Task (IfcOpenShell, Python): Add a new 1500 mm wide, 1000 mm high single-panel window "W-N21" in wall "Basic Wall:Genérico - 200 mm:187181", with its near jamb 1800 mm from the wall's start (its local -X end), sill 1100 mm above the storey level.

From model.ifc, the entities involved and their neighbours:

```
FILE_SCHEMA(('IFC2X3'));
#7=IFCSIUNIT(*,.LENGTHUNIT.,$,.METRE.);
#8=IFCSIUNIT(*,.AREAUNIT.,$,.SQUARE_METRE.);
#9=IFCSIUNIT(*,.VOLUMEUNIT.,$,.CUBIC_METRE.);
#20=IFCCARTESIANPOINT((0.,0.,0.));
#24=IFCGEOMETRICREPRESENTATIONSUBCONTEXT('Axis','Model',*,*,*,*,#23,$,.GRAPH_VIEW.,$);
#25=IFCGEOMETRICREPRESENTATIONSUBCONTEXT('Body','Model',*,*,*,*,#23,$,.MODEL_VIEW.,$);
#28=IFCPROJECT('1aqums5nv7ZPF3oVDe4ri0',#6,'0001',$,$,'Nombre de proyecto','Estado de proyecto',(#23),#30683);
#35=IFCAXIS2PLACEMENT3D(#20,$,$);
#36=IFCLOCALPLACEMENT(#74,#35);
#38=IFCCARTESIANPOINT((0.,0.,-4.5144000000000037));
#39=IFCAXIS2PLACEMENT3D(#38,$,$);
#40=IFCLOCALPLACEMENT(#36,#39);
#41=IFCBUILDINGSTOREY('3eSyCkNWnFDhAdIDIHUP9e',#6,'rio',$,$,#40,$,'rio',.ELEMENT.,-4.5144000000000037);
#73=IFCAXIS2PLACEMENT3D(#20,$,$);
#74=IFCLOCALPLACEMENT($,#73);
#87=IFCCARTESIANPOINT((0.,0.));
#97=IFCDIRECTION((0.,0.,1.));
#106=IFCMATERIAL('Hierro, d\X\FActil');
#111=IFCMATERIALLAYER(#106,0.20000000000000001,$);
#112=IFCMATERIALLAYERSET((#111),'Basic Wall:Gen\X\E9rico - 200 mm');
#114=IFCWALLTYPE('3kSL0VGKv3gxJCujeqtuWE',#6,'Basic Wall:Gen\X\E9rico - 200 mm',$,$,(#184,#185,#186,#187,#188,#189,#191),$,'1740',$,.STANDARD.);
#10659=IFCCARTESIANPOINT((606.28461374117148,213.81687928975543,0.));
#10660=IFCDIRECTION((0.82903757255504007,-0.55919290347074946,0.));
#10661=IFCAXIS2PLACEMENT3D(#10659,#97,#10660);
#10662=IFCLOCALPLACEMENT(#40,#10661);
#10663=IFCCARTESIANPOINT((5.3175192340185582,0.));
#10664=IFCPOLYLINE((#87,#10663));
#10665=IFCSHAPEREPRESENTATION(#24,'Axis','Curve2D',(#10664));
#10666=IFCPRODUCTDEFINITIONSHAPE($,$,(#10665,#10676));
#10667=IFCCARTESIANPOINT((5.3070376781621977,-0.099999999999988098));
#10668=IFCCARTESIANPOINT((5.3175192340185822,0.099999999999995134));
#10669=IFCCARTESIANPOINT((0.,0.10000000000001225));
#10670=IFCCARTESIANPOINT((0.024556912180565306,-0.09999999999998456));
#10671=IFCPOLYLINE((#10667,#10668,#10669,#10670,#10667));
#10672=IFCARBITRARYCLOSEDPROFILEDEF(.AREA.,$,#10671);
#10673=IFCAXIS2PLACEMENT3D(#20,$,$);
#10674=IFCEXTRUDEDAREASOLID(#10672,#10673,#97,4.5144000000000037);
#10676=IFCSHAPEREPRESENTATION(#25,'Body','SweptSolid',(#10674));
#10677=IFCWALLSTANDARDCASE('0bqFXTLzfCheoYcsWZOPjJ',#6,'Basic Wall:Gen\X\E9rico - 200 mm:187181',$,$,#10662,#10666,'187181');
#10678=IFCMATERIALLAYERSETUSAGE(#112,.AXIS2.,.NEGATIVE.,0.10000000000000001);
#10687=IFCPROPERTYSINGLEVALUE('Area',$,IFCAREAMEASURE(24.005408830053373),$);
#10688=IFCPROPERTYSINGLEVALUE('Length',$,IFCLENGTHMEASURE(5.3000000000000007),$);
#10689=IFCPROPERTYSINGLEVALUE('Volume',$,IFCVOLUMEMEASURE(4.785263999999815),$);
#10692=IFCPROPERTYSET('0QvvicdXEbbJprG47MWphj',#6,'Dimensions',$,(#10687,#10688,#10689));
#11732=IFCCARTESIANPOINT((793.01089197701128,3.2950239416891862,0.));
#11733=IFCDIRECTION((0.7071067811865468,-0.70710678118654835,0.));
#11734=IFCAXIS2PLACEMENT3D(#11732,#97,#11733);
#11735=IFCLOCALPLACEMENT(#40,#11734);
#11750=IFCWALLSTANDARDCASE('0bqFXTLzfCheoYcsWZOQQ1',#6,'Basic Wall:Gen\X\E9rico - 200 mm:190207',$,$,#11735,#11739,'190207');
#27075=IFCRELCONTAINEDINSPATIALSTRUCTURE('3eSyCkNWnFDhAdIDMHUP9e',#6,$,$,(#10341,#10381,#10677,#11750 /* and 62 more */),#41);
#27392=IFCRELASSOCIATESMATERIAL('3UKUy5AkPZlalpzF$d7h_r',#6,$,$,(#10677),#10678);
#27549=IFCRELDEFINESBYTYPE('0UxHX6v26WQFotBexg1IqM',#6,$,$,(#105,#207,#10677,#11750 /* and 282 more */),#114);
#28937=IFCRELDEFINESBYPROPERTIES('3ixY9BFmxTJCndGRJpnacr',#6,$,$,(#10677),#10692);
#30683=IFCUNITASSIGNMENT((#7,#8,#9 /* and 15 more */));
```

```python
import numpy as np
import ifcopenshell
import ifcopenshell.api.feature
import ifcopenshell.api.geometry
import ifcopenshell.api.pset
import ifcopenshell.api.root
import ifcopenshell.api.spatial
import ifcopenshell.api.type
import ifcopenshell.geom
import ifcopenshell.util.element
import ifcopenshell.util.placement
import ifcopenshell.util.representation
import ifcopenshell.util.shape
import ifcopenshell.util.unit

model = ifcopenshell.open("model.ifc")
unit_scale = ifcopenshell.util.unit.calculate_unit_scale(model)
area_scale = ifcopenshell.util.unit.calculate_unit_scale(model, "AREAUNIT")
volume_scale = ifcopenshell.util.unit.calculate_unit_scale(model, "VOLUMEUNIT")
settings = ifcopenshell.geom.settings()


def volume(element):
    """Net volume in cubic metres, openings subtracted."""
    shape = ifcopenshell.geom.create_shape(settings, element)
    return ifcopenshell.util.shape.get_volume(shape.geometry)


wall = model.by_guid("0bqFXTLzfCheoYcsWZOPjJ")
storey = ifcopenshell.util.element.get_container(wall, ifc_class="IfcBuildingStorey")
context = ifcopenshell.util.representation.get_context(model, "Model", "Body", "MODEL_VIEW")
before = volume(wall)

width, height, from_end, sill = 1.5, 1, 1.8, 1.1  # metres

# The wall runs along its own X axis, and the end named is its -X end.
wall_shape = ifcopenshell.geom.create_shape(settings, wall)
x, y, z = ifcopenshell.util.shape.get_vertices(wall_shape.geometry).T
start = x.min() + from_end
face, thickness = float(y.min()), float(y.max() - y.min())
wall_matrix = ifcopenshell.util.placement.get_local_placement(wall.ObjectPlacement)
level = ifcopenshell.util.placement.get_local_placement(storey.ObjectPlacement)[2, 3]


def in_wall(x, y):
    """Placement at x, y metres in the wall's axes, at sill height."""
    matrix = wall_matrix.copy()
    matrix[:, 3] = wall_matrix @ np.array([x / unit_scale, y / unit_scale, 0.0, 1.0])
    matrix[2, 3] = level + sill / unit_scale
    return matrix


# Opening: a box that overshoots both wall faces by 50 mm.
opening = ifcopenshell.api.root.create_entity(model, ifc_class="IfcOpeningElement")
box = ifcopenshell.api.geometry.add_wall_representation(
    model, context=context, length=width, height=height, thickness=thickness + 0.1
)
ifcopenshell.api.geometry.assign_representation(model, product=opening, representation=box)
ifcopenshell.api.geometry.edit_object_placement(model, product=opening, matrix=in_wall(start, face - 0.05), is_si=False)
ifcopenshell.api.feature.add_feature(model, feature=opening, element=wall)

window = ifcopenshell.api.root.create_entity(model, ifc_class="IfcWindow", name="W-N21")
window.OverallWidth, window.OverallHeight = width / unit_scale, height / unit_scale
body = ifcopenshell.api.geometry.add_window_representation(
    model,
    context=context,
    overall_width=window.OverallWidth,
    overall_height=window.OverallHeight,
    partition_type="SINGLE_PANEL",
)
ifcopenshell.api.geometry.assign_representation(model, product=window, representation=body)
ifcopenshell.api.spatial.assign_container(model, products=[window], relating_structure=storey)
fills = ifcopenshell.api.feature.add_filling(model, opening=opening, element=window)
fills.OwnerHistory = window.OwnerHistory  # required in IFC2X3

# IFC2X3 keeps the operation on the window style.
style = ifcopenshell.api.root.create_entity(model, ifc_class="IfcWindowStyle", name="W-N21")
style.OperationType, style.ConstructionType = "SINGLE_PANEL", "NOTDEFINED"
style.ParameterTakesPrecedence = style.Sizeable = False
ifcopenshell.api.type.assign_type(model, related_objects=[window], relating_type=style)

# Centre the window in the wall's thickness.
ifcopenshell.api.geometry.edit_object_placement(model, product=window, matrix=in_wall(start, face), is_si=False)
window_shape = ifcopenshell.geom.create_shape(settings, window)
depth = ifcopenshell.util.shape.get_vertices(window_shape.geometry)[:, 1]
offset = face + thickness / 2 - (depth.min() + depth.max()) / 2
ifcopenshell.api.geometry.edit_object_placement(model, product=window, matrix=in_wall(start, offset), is_si=False)

after = volume(wall)

# Update the wall's stored quantities.
pset = model.by_id(ifcopenshell.util.element.get_pset(wall, "Dimensions", should_inherit=False)["id"])
ifcopenshell.api.pset.edit_pset(model, pset=pset, properties={
    "Area": model.create_entity("IfcAreaMeasure", after / thickness / area_scale),
    "Volume": model.create_entity("IfcVolumeMeasure", after / volume_scale),
})

print(f"wall volume {before:.3f} -> {after:.3f} m3")

model.write("model_edited.ifc")
```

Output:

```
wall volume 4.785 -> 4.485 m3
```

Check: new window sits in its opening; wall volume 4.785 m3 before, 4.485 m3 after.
